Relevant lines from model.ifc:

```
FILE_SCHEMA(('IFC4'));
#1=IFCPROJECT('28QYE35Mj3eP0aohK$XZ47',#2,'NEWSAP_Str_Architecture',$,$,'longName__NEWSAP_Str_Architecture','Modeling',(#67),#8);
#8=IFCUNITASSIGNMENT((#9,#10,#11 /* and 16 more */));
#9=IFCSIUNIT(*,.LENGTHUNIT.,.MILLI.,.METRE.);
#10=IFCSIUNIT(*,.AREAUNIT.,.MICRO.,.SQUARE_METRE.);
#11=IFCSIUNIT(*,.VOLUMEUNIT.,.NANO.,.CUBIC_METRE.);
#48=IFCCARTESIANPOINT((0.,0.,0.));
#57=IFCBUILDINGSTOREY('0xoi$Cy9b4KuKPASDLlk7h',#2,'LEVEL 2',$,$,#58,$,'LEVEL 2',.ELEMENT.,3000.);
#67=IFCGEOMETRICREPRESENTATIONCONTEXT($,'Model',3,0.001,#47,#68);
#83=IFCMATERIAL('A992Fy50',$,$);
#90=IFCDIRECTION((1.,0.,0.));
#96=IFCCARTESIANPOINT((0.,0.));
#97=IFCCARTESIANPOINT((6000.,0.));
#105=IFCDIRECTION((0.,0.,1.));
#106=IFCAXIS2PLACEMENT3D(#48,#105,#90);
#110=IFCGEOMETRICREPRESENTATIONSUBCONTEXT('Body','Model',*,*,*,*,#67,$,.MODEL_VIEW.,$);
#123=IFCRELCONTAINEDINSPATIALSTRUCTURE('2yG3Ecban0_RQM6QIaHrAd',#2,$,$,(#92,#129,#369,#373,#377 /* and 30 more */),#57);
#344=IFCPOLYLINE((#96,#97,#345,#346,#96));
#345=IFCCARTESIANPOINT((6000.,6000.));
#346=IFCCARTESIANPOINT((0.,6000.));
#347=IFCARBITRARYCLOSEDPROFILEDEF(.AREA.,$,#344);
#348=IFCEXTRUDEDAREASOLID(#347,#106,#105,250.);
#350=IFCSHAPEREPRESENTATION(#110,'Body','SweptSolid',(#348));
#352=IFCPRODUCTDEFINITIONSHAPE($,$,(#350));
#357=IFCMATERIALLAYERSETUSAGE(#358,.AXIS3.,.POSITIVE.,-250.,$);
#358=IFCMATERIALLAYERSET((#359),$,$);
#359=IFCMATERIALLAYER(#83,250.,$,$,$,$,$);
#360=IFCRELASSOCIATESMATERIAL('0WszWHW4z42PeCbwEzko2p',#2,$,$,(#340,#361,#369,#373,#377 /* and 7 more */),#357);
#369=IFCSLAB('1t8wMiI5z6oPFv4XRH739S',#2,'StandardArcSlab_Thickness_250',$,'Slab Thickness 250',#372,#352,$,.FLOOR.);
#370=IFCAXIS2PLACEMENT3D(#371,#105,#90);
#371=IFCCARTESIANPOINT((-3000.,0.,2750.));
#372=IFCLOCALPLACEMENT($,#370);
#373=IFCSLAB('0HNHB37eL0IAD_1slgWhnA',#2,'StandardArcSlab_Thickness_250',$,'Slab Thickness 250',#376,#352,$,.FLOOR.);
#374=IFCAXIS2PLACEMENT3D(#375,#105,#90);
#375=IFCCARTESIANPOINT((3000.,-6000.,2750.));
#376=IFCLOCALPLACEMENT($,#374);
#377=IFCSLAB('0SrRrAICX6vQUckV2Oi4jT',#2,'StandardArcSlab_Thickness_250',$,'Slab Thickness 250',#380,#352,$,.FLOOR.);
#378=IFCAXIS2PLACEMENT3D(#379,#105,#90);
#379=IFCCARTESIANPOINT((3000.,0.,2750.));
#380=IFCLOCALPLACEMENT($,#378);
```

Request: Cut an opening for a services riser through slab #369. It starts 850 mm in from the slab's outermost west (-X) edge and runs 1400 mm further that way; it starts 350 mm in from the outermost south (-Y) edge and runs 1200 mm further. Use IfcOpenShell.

```python
import numpy as np
import ifcopenshell
import ifcopenshell.api.feature
import ifcopenshell.api.geometry
import ifcopenshell.api.root
import ifcopenshell.geom
import ifcopenshell.util.placement
import ifcopenshell.util.representation
import ifcopenshell.util.shape
import ifcopenshell.util.unit

model = ifcopenshell.open("model.ifc")
unit_scale = ifcopenshell.util.unit.calculate_unit_scale(model)
settings = ifcopenshell.geom.settings()


def volume(element):
    """Net volume in cubic metres, openings subtracted."""
    shape = ifcopenshell.geom.create_shape(settings, element)
    return ifcopenshell.util.shape.get_volume(shape.geometry)


slab = model.by_id(369)
before = volume(slab)

# Extent in the slab's own axes, in metres. The edges named are its -X and -Y sides.
slab_shape = ifcopenshell.geom.create_shape(settings, slab)
vertices = ifcopenshell.util.shape.get_vertices(slab_shape.geometry)
x_min, y_min, bottom = vertices.min(axis=0)
top = vertices[:, 2].max()

opening = ifcopenshell.api.root.create_entity(model, ifc_class="IfcOpeningElement", name="Services riser opening", predefined_type="OPENING")
context = ifcopenshell.util.representation.get_context(model, "Model", "Body", "MODEL_VIEW")
width, depth = 1.4, 1.2
outline = [(0.0, 0.0), (width, 0.0), (width, depth), (0.0, depth), (0.0, 0.0)]
# Overshoot both faces by 50 mm so the cut is clean.
shape = ifcopenshell.api.geometry.add_slab_representation(
    model, context=context, depth=top - bottom + 0.1, polyline=outline
)
ifcopenshell.api.geometry.assign_representation(model, product=opening, representation=shape)

matrix = ifcopenshell.util.placement.get_local_placement(slab.ObjectPlacement)
matrix[:, 3] = matrix @ np.append(np.array([x_min + 0.85, y_min + 0.35, bottom - 0.05]) / unit_scale, 1.0)
ifcopenshell.api.geometry.edit_object_placement(model, product=opening, matrix=matrix, is_si=False)
ifcopenshell.api.feature.add_feature(model, feature=opening, element=slab)

after = volume(slab)

print(f"slab volume {before:.3f} -> {after:.3f} m3")

model.write("model_edited.ifc")
```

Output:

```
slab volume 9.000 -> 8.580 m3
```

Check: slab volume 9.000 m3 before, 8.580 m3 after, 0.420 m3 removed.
